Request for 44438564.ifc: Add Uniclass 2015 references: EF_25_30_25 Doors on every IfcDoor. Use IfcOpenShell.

First a look at what the model holds.

```python
import ifcopenshell

model = ifcopenshell.open("44438564.ifc")
print(model.schema)
print("classifications:", [c.Name for c in model.by_type("IfcClassification")])
for ifc_class in ("IfcDoor", "IfcRoof", "IfcStair", "IfcWall", "IfcWindow"):
    print(ifc_class, len(model.by_type(ifc_class)))
```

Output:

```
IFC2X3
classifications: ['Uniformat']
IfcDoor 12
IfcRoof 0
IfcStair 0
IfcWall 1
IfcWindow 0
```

```python
import ifcopenshell
import ifcopenshell.api.classification

model = ifcopenshell.open("44438564.ifc")

# IFC2X3 requires Source and Edition and has no link from the project to the system.
system = model.create_entity("IfcClassification", Source="NBS", Edition="2015", Name="Uniclass 2015")

codes = {
    "IfcDoor": ("EF_25_30_25", "Doors"),
}
for ifc_class, (code, name) in codes.items():
    products = model.by_type(ifc_class)
    ifcopenshell.api.classification.add_reference(
        model, products=products, classification=system, identification=code, name=name
    )
    print(code, len(products))

model.write("44438564_rev.ifc")
```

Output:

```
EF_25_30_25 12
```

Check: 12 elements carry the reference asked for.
